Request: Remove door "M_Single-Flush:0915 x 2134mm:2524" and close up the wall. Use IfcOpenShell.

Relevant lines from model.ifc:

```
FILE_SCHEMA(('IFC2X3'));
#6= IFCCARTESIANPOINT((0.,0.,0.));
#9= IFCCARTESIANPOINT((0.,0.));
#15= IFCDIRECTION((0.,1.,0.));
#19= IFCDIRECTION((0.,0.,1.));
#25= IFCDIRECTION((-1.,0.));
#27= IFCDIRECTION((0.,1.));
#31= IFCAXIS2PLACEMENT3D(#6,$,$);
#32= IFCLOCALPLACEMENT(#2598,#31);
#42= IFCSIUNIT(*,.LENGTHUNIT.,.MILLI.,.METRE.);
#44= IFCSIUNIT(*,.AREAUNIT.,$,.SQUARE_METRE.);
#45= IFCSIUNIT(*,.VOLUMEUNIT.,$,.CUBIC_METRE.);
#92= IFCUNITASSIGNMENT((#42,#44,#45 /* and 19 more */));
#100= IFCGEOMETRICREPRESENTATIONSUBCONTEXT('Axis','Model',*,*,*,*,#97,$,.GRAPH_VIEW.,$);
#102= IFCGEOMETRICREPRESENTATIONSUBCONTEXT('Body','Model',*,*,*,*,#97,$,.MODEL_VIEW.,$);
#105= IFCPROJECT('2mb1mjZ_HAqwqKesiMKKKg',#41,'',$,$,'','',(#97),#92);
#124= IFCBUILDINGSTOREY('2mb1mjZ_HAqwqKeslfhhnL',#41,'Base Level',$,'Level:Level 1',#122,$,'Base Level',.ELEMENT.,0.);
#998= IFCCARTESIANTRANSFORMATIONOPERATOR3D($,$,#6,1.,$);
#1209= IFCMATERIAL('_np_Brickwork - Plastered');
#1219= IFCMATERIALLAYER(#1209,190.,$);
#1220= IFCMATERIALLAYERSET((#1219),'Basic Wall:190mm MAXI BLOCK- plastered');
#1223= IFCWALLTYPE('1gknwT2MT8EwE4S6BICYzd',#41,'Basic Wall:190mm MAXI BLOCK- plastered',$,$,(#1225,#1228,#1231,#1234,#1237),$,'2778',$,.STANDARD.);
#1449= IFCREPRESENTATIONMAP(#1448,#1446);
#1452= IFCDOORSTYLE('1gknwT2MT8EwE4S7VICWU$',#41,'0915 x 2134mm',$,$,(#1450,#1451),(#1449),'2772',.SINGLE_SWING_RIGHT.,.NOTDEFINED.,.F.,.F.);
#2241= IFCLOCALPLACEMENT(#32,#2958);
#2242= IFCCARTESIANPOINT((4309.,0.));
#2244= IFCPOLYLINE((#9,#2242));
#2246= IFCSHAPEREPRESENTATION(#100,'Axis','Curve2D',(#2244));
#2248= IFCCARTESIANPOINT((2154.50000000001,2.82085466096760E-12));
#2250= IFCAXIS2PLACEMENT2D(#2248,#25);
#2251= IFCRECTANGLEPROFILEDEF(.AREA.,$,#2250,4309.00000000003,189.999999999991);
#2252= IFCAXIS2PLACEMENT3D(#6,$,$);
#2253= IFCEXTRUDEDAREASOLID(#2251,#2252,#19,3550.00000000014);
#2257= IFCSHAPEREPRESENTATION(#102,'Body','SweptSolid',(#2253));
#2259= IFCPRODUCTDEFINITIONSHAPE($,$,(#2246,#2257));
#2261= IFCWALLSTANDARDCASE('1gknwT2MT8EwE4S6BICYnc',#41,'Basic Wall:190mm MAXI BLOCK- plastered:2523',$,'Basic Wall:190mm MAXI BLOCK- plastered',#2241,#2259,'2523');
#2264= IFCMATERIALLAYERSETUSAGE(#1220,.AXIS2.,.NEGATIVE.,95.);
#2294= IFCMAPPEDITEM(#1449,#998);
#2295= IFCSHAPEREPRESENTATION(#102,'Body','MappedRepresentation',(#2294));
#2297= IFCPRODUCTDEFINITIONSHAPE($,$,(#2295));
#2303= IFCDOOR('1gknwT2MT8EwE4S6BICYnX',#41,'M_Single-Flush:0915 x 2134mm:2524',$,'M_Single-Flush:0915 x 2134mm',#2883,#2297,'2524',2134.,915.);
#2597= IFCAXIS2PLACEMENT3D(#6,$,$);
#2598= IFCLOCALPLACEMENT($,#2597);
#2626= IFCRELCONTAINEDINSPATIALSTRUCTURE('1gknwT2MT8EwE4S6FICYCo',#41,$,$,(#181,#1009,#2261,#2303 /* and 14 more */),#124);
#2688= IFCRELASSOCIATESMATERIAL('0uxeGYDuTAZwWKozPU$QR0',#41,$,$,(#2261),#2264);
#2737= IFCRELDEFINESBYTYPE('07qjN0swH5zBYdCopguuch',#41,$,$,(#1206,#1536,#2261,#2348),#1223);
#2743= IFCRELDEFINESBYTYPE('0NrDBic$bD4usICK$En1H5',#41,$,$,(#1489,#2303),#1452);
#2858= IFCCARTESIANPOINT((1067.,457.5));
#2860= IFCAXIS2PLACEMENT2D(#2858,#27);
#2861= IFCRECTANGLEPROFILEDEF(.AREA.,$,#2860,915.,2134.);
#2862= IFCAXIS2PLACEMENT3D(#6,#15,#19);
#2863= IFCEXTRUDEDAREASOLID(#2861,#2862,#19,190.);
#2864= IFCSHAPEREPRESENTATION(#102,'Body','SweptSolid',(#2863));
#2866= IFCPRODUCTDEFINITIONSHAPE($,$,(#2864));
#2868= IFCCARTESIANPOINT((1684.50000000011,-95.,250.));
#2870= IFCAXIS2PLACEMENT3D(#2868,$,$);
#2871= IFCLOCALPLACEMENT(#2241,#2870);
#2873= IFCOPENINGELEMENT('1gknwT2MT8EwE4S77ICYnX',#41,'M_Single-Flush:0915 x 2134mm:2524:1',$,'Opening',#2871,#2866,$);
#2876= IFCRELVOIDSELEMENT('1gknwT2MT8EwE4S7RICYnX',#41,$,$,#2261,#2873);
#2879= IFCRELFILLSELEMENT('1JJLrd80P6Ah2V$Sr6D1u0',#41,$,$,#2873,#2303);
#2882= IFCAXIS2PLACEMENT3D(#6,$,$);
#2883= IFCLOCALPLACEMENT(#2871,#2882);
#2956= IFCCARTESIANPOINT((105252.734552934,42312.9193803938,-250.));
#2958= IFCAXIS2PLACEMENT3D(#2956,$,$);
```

```python
import ifcopenshell
import ifcopenshell.api.feature
import ifcopenshell.api.root
import ifcopenshell.geom
import ifcopenshell.util.shape

model = ifcopenshell.open("model.ifc")
settings = ifcopenshell.geom.settings()


def volume(element):
    """Net volume in cubic metres, openings subtracted."""
    shape = ifcopenshell.geom.create_shape(settings, element)
    return ifcopenshell.util.shape.get_volume(shape.geometry)


door = model.by_guid("1gknwT2MT8EwE4S6BICYnX")
opening = door.FillsVoids[0].RelatingOpeningElement
wall = opening.VoidsElements[0].RelatingBuildingElement
before = volume(wall)

ifcopenshell.api.root.remove_product(model, product=door)
ifcopenshell.api.feature.remove_feature(model, feature=opening)

after = volume(wall)

print(f"wall volume {before:.3f} -> {after:.3f} m3")

model.write("model_v2.ifc")
```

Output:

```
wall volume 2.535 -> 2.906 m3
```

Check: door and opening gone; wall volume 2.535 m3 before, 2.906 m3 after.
